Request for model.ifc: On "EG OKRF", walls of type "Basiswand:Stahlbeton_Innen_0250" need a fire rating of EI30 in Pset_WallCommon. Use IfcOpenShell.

First a look at what the model holds.

```python
import ifcopenshell
import ifcopenshell.util.element

model = ifcopenshell.open("model.ifc")
print(model.schema)
storey = next(s for s in model.by_type("IfcBuildingStorey") if s.Name == "EG OKRF")
walls = [e for e in ifcopenshell.util.element.get_decomposition(storey) if e.is_a("IfcWall")]
seen = {}
for e in walls:
    element_type = ifcopenshell.util.element.get_type(e)
    key = (element_type.Name if element_type != e and element_type else None, ifcopenshell.util.element.get_pset(e, "Pset_WallCommon", "FireRating"))
    seen[key] = seen.get(key, 0) + 1
for (name, value), count in sorted(seen.items(), key=str):
    print(count, "x", name, "|", value)
```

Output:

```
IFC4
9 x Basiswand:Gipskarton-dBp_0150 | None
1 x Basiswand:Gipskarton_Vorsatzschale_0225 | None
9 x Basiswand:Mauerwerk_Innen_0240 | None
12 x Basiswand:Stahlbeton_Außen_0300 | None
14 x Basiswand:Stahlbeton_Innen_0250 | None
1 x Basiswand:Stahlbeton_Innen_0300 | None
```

```python
import ifcopenshell
import ifcopenshell.api.pset
import ifcopenshell.util.element

model = ifcopenshell.open("model.ifc")

storey = next(s for s in model.by_type("IfcBuildingStorey") if s.Name == "EG OKRF")
walls = [e for e in ifcopenshell.util.element.get_decomposition(storey) if e.is_a("IfcWall")]

count = 0
for e in walls:
    element_type = ifcopenshell.util.element.get_type(e)
    if element_type in (None, e) or element_type.Name != "Basiswand:Stahlbeton_Innen_0250":
        continue
    # add_pset returns the element's existing set when there is one.
    pset = ifcopenshell.api.pset.add_pset(model, product=e, name="Pset_WallCommon")
    ifcopenshell.api.pset.edit_pset(model, pset=pset, properties={"FireRating": "EI30"})
    count += 1

print(count, "walls updated")

model.write("model_updated.ifc")
```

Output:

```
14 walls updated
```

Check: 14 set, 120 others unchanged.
